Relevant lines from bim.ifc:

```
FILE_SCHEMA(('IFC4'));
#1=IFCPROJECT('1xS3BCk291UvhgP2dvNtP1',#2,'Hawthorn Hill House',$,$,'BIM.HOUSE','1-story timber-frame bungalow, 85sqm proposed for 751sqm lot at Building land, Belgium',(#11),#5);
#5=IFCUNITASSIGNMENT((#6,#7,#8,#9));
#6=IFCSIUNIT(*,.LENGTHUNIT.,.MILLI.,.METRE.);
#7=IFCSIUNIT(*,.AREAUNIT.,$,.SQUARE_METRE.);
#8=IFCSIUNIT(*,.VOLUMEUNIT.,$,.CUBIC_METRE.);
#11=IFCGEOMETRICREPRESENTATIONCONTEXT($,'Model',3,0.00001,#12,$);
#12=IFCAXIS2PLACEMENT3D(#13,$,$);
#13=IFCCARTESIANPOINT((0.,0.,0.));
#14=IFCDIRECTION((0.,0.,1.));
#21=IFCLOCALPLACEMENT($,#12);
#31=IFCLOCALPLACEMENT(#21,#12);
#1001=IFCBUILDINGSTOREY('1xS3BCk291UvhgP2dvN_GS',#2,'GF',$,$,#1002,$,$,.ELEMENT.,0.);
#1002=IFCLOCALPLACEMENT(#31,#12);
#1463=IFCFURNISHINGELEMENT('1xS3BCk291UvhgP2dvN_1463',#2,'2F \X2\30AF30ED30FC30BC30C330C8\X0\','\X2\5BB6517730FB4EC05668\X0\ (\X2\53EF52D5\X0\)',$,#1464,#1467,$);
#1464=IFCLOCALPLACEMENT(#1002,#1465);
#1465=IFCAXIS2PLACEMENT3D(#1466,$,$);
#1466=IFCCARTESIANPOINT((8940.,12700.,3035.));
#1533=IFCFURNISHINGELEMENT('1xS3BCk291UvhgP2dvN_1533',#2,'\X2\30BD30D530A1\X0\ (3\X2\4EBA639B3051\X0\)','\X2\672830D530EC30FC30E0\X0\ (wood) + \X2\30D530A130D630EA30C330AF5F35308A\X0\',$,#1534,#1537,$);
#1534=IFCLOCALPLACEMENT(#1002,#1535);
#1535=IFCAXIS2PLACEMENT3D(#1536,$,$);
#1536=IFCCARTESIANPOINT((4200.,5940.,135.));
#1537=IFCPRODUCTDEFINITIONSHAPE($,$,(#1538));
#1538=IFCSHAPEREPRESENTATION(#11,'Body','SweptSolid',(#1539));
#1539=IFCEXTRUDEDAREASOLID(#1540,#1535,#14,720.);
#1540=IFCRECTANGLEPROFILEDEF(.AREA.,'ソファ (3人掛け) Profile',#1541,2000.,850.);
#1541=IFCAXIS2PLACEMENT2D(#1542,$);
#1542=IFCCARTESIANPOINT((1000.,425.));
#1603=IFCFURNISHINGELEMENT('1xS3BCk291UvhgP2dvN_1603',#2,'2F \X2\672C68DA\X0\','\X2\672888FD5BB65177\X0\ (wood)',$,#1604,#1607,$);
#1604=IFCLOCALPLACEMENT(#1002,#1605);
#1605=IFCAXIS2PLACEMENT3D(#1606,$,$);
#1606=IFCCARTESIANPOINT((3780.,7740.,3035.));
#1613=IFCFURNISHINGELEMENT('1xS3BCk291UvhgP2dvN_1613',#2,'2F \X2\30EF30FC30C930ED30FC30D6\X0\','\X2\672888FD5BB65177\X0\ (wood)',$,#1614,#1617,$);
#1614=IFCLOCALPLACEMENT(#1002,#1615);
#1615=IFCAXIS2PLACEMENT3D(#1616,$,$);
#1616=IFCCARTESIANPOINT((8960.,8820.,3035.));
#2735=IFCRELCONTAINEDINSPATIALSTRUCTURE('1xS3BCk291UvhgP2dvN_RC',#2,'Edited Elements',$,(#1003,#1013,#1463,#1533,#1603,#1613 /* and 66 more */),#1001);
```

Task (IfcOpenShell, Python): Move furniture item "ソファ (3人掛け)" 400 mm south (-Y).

```python
import ifcopenshell
import ifcopenshell.api.geometry
import ifcopenshell.util.placement
import ifcopenshell.util.unit

model = ifcopenshell.open("bim.ifc")
unit_scale = ifcopenshell.util.unit.calculate_unit_scale(model)

item = model.by_id(1533)
matrix = ifcopenshell.util.placement.get_local_placement(item.ObjectPlacement)
matrix[1, 3] -= 0.4 / unit_scale
ifcopenshell.api.geometry.edit_object_placement(model, product=item, matrix=matrix, is_si=False)

print(ifcopenshell.util.placement.get_local_placement(item.ObjectPlacement).round(3) + 0.0)

model.write("bim_rev.ifc")
```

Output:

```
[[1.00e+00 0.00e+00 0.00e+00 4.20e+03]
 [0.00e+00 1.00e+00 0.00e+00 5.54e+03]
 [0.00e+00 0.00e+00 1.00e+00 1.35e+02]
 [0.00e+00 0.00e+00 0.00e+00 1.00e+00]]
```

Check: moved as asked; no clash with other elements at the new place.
